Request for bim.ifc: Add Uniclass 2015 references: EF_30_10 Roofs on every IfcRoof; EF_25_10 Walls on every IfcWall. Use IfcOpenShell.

First a look at what the model holds.

```python
import ifcopenshell

model = ifcopenshell.open("bim.ifc")
print(model.schema)
print("classifications:", [c.Name for c in model.by_type("IfcClassification")])
for ifc_class in ("IfcDoor", "IfcRoof", "IfcStair", "IfcWall", "IfcWindow"):
    print(ifc_class, len(model.by_type(ifc_class)))
```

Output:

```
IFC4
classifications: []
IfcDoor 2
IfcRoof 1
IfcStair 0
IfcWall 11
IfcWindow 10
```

```python
import ifcopenshell
import ifcopenshell.api.classification

model = ifcopenshell.open("bim.ifc")

system = ifcopenshell.api.classification.add_classification(model, classification="Uniclass 2015")

codes = {
    "IfcRoof": ("EF_30_10", "Roofs"),
    "IfcWall": ("EF_25_10", "Walls"),
}
for ifc_class, (code, name) in codes.items():
    products = model.by_type(ifc_class)
    ifcopenshell.api.classification.add_reference(
        model, products=products, classification=system, identification=code, name=name
    )
    print(code, len(products))

model.write("bim_updated.ifc")
```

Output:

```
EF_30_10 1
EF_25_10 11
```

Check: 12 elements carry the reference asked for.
